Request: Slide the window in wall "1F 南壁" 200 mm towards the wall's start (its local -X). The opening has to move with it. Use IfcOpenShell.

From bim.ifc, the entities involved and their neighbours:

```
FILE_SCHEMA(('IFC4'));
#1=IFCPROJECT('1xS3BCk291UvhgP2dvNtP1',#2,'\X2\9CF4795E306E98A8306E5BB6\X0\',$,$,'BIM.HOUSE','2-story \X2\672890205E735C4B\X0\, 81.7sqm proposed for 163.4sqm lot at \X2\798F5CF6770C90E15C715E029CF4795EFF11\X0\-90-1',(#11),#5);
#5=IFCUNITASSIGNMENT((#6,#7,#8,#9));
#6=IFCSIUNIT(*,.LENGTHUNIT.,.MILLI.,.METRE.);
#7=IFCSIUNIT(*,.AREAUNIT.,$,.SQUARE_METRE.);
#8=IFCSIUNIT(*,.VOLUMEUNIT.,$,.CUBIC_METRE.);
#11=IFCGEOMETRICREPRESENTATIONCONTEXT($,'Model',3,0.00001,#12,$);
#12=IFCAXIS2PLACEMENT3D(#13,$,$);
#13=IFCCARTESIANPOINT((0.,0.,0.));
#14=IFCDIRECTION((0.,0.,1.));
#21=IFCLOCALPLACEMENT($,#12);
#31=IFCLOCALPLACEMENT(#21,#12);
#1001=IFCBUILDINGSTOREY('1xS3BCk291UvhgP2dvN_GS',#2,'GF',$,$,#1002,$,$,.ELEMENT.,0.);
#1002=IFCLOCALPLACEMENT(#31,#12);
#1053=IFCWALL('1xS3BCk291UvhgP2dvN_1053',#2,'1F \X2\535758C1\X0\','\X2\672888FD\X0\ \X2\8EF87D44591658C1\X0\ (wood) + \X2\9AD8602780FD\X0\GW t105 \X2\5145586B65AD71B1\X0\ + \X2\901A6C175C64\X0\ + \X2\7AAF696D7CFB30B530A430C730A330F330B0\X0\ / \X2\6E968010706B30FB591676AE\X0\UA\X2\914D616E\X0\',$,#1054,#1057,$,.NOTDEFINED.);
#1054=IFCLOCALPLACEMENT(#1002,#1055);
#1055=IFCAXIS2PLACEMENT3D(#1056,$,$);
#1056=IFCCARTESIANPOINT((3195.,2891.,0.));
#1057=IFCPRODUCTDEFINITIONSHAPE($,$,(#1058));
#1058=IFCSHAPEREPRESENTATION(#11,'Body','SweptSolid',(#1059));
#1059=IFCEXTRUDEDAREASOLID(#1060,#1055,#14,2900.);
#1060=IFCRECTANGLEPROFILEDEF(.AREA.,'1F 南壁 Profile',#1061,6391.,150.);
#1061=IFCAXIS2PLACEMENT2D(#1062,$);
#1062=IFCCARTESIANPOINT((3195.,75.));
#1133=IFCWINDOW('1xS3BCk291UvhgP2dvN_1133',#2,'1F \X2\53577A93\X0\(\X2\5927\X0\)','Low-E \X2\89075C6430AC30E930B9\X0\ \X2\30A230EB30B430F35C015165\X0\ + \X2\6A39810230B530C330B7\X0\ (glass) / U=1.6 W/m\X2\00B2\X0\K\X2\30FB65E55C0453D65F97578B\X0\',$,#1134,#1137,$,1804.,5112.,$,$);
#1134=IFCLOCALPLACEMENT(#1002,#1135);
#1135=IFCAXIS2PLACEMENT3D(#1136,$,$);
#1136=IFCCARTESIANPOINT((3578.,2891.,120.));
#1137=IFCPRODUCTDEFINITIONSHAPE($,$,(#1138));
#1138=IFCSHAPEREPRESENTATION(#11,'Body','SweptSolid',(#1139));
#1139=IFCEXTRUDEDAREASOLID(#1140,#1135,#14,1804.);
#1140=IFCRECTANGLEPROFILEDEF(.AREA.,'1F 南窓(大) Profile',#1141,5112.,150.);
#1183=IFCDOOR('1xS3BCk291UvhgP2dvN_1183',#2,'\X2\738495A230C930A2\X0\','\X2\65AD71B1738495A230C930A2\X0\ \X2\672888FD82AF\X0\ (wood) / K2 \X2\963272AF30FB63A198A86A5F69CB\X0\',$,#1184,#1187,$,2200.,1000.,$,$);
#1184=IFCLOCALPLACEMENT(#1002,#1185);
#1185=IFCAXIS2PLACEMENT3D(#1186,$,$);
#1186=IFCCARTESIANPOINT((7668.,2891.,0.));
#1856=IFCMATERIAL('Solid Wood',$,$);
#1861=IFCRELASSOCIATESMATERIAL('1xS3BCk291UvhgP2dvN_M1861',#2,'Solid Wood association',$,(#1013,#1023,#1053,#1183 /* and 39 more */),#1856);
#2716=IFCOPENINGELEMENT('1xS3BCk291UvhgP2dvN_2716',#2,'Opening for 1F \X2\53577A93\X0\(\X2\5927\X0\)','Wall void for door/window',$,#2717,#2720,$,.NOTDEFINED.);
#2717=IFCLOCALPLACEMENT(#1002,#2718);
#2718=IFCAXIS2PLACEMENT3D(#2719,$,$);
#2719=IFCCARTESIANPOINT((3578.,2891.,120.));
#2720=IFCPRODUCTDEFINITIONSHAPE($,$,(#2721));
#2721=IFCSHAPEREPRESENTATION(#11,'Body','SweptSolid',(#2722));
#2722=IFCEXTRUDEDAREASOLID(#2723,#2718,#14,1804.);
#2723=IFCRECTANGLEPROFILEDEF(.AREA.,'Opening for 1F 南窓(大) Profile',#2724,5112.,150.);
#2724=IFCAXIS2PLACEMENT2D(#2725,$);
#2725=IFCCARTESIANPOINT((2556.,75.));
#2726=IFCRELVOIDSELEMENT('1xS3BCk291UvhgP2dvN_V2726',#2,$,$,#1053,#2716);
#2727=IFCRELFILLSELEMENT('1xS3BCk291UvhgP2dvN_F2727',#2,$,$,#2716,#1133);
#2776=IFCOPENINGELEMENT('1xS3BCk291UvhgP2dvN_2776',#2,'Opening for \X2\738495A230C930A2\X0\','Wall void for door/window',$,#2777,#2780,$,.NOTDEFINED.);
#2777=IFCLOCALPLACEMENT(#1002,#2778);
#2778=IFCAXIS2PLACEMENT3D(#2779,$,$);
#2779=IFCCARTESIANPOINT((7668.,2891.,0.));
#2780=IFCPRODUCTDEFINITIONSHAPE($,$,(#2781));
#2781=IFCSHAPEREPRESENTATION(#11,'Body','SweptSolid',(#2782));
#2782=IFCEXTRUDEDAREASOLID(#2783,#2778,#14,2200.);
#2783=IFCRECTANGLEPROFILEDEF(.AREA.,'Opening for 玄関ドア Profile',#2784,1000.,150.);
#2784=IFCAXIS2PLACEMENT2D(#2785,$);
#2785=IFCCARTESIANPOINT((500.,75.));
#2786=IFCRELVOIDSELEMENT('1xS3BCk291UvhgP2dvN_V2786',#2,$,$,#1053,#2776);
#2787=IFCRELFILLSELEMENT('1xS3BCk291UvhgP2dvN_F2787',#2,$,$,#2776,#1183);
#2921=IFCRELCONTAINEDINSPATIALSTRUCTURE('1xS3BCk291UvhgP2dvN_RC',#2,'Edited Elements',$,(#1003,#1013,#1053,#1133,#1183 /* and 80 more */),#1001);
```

```python
import ifcopenshell
import ifcopenshell.api.geometry
import ifcopenshell.util.placement
import ifcopenshell.util.unit

model = ifcopenshell.open("bim.ifc")
unit_scale = ifcopenshell.util.unit.calculate_unit_scale(model)

window = model.by_guid("1xS3BCk291UvhgP2dvN_1133")
opening = window.FillsVoids[0].RelatingOpeningElement
wall = opening.VoidsElements[0].RelatingBuildingElement

wall_matrix = ifcopenshell.util.placement.get_local_placement(wall.ObjectPlacement)
shift = wall_matrix[:3, 0] * -0.2 / unit_scale
before = ifcopenshell.util.placement.get_local_placement(window.ObjectPlacement)[:3, 3].copy()

# The window is not placed relative to its opening, so move both.
for product in (opening, window):
    matrix = ifcopenshell.util.placement.get_local_placement(product.ObjectPlacement)
    matrix[:3, 3] += shift
    ifcopenshell.api.geometry.edit_object_placement(model, product=product, matrix=matrix, is_si=False)

after = ifcopenshell.util.placement.get_local_placement(window.ObjectPlacement)[:3, 3]
print("window moved by", (after - before).round(3) + 0.0)

model.write("bim_updated.ifc")
```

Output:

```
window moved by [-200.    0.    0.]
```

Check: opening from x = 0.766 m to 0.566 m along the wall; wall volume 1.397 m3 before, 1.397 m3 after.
